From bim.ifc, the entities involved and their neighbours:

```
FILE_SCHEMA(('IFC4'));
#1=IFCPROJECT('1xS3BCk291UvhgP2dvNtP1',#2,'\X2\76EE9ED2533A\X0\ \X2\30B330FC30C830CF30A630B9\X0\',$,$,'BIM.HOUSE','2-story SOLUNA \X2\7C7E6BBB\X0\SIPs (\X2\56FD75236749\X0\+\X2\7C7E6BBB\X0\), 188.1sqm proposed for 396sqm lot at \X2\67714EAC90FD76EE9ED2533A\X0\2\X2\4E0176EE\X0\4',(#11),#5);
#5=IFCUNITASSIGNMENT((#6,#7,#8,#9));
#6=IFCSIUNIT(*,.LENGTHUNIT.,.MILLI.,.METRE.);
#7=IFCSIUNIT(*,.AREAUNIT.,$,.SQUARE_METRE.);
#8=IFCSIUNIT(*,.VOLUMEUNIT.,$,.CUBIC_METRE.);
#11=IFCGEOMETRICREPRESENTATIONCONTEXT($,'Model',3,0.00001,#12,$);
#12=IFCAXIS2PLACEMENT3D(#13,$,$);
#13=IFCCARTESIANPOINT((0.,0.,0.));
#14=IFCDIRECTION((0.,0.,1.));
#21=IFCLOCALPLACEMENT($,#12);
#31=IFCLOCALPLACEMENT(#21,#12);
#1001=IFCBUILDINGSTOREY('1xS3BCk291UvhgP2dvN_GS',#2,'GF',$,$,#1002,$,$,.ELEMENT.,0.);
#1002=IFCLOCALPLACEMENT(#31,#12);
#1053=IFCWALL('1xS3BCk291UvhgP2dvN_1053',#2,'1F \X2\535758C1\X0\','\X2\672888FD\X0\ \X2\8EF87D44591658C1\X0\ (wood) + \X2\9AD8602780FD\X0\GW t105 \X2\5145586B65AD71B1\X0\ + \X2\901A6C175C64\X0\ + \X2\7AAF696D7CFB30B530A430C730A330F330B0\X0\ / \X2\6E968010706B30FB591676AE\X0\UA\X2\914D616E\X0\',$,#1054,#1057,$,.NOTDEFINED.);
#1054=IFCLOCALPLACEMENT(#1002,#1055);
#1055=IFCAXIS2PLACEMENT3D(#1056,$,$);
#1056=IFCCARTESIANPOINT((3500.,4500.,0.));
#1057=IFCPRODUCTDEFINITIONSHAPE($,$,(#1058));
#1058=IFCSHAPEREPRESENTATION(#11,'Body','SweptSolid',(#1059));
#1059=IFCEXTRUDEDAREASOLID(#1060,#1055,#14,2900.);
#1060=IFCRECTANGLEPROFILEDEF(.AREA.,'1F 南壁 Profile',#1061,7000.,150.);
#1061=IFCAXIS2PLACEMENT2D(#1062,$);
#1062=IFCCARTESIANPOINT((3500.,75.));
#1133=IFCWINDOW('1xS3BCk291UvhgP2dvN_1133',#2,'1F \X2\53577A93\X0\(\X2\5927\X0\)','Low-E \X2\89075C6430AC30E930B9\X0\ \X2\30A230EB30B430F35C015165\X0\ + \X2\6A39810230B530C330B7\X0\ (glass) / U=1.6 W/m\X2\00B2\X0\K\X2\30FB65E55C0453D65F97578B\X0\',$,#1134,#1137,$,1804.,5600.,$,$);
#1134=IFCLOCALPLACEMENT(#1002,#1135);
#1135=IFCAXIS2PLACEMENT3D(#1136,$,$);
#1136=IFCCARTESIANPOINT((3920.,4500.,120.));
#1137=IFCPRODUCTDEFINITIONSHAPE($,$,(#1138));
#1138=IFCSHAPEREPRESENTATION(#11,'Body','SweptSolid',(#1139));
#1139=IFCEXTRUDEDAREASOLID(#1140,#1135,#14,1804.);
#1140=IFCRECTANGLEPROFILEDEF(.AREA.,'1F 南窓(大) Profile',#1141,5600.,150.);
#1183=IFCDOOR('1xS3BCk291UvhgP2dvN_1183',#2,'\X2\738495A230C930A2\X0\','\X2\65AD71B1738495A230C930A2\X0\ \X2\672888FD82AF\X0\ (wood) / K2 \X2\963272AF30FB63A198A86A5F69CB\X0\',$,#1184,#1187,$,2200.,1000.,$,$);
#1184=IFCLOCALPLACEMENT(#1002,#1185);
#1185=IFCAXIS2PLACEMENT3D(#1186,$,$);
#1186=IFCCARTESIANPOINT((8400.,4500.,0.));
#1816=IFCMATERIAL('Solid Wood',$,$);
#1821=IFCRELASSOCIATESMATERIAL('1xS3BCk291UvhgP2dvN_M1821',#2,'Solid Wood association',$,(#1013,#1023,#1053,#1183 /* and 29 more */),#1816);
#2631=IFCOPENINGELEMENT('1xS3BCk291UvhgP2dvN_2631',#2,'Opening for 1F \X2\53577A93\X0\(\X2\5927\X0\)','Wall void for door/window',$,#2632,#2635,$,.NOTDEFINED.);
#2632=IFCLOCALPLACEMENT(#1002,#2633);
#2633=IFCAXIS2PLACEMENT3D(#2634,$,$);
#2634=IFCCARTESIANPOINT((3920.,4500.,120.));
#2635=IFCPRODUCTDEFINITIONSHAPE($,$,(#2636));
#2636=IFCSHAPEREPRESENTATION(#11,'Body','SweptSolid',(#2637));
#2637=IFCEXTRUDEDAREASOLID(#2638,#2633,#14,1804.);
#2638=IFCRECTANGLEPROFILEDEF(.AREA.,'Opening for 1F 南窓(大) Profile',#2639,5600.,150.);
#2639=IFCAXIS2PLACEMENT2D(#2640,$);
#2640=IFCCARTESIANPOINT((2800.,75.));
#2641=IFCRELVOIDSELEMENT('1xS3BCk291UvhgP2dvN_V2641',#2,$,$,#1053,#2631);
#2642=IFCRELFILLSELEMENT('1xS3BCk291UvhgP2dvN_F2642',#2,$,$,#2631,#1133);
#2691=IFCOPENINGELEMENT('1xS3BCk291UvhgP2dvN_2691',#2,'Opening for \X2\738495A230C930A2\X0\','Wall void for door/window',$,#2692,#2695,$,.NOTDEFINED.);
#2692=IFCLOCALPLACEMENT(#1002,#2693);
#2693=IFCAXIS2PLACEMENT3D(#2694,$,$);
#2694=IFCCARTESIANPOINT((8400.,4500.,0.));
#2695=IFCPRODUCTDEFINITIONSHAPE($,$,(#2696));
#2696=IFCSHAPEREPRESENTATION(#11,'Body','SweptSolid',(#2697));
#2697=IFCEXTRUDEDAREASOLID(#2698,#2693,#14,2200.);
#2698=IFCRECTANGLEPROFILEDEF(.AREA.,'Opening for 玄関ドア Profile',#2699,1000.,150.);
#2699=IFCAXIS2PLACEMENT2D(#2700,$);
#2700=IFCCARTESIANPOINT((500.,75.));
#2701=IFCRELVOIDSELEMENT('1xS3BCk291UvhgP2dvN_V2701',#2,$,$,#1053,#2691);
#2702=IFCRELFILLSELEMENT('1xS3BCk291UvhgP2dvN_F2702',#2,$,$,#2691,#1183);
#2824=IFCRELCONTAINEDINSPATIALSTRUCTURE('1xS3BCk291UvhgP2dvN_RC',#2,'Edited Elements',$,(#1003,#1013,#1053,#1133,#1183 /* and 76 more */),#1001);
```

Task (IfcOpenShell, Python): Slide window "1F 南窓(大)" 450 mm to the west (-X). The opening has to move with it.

```python
import ifcopenshell
import ifcopenshell.api.geometry
import ifcopenshell.util.placement

model = ifcopenshell.open("bim.ifc")

window = model.by_id(1133)
opening = window.FillsVoids[0].RelatingOpeningElement
wall = opening.VoidsElements[0].RelatingBuildingElement

wall_matrix = ifcopenshell.util.placement.get_local_placement(wall.ObjectPlacement)
shift = wall_matrix[:3, 0] * -450.0
before = ifcopenshell.util.placement.get_local_placement(window.ObjectPlacement)[:3, 3].copy()

# The window is not placed relative to its opening, so move both.
for product in (opening, window):
    matrix = ifcopenshell.util.placement.get_local_placement(product.ObjectPlacement)
    matrix[:3, 3] += shift
    ifcopenshell.api.geometry.edit_object_placement(model, product=product, matrix=matrix, is_si=False)

after = ifcopenshell.util.placement.get_local_placement(window.ObjectPlacement)[:3, 3]
print("window moved by", (after - before).round(3) + 0.0)

model.write("bim_v2.ifc")
```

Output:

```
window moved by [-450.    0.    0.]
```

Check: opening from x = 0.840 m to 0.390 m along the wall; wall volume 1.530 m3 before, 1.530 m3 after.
